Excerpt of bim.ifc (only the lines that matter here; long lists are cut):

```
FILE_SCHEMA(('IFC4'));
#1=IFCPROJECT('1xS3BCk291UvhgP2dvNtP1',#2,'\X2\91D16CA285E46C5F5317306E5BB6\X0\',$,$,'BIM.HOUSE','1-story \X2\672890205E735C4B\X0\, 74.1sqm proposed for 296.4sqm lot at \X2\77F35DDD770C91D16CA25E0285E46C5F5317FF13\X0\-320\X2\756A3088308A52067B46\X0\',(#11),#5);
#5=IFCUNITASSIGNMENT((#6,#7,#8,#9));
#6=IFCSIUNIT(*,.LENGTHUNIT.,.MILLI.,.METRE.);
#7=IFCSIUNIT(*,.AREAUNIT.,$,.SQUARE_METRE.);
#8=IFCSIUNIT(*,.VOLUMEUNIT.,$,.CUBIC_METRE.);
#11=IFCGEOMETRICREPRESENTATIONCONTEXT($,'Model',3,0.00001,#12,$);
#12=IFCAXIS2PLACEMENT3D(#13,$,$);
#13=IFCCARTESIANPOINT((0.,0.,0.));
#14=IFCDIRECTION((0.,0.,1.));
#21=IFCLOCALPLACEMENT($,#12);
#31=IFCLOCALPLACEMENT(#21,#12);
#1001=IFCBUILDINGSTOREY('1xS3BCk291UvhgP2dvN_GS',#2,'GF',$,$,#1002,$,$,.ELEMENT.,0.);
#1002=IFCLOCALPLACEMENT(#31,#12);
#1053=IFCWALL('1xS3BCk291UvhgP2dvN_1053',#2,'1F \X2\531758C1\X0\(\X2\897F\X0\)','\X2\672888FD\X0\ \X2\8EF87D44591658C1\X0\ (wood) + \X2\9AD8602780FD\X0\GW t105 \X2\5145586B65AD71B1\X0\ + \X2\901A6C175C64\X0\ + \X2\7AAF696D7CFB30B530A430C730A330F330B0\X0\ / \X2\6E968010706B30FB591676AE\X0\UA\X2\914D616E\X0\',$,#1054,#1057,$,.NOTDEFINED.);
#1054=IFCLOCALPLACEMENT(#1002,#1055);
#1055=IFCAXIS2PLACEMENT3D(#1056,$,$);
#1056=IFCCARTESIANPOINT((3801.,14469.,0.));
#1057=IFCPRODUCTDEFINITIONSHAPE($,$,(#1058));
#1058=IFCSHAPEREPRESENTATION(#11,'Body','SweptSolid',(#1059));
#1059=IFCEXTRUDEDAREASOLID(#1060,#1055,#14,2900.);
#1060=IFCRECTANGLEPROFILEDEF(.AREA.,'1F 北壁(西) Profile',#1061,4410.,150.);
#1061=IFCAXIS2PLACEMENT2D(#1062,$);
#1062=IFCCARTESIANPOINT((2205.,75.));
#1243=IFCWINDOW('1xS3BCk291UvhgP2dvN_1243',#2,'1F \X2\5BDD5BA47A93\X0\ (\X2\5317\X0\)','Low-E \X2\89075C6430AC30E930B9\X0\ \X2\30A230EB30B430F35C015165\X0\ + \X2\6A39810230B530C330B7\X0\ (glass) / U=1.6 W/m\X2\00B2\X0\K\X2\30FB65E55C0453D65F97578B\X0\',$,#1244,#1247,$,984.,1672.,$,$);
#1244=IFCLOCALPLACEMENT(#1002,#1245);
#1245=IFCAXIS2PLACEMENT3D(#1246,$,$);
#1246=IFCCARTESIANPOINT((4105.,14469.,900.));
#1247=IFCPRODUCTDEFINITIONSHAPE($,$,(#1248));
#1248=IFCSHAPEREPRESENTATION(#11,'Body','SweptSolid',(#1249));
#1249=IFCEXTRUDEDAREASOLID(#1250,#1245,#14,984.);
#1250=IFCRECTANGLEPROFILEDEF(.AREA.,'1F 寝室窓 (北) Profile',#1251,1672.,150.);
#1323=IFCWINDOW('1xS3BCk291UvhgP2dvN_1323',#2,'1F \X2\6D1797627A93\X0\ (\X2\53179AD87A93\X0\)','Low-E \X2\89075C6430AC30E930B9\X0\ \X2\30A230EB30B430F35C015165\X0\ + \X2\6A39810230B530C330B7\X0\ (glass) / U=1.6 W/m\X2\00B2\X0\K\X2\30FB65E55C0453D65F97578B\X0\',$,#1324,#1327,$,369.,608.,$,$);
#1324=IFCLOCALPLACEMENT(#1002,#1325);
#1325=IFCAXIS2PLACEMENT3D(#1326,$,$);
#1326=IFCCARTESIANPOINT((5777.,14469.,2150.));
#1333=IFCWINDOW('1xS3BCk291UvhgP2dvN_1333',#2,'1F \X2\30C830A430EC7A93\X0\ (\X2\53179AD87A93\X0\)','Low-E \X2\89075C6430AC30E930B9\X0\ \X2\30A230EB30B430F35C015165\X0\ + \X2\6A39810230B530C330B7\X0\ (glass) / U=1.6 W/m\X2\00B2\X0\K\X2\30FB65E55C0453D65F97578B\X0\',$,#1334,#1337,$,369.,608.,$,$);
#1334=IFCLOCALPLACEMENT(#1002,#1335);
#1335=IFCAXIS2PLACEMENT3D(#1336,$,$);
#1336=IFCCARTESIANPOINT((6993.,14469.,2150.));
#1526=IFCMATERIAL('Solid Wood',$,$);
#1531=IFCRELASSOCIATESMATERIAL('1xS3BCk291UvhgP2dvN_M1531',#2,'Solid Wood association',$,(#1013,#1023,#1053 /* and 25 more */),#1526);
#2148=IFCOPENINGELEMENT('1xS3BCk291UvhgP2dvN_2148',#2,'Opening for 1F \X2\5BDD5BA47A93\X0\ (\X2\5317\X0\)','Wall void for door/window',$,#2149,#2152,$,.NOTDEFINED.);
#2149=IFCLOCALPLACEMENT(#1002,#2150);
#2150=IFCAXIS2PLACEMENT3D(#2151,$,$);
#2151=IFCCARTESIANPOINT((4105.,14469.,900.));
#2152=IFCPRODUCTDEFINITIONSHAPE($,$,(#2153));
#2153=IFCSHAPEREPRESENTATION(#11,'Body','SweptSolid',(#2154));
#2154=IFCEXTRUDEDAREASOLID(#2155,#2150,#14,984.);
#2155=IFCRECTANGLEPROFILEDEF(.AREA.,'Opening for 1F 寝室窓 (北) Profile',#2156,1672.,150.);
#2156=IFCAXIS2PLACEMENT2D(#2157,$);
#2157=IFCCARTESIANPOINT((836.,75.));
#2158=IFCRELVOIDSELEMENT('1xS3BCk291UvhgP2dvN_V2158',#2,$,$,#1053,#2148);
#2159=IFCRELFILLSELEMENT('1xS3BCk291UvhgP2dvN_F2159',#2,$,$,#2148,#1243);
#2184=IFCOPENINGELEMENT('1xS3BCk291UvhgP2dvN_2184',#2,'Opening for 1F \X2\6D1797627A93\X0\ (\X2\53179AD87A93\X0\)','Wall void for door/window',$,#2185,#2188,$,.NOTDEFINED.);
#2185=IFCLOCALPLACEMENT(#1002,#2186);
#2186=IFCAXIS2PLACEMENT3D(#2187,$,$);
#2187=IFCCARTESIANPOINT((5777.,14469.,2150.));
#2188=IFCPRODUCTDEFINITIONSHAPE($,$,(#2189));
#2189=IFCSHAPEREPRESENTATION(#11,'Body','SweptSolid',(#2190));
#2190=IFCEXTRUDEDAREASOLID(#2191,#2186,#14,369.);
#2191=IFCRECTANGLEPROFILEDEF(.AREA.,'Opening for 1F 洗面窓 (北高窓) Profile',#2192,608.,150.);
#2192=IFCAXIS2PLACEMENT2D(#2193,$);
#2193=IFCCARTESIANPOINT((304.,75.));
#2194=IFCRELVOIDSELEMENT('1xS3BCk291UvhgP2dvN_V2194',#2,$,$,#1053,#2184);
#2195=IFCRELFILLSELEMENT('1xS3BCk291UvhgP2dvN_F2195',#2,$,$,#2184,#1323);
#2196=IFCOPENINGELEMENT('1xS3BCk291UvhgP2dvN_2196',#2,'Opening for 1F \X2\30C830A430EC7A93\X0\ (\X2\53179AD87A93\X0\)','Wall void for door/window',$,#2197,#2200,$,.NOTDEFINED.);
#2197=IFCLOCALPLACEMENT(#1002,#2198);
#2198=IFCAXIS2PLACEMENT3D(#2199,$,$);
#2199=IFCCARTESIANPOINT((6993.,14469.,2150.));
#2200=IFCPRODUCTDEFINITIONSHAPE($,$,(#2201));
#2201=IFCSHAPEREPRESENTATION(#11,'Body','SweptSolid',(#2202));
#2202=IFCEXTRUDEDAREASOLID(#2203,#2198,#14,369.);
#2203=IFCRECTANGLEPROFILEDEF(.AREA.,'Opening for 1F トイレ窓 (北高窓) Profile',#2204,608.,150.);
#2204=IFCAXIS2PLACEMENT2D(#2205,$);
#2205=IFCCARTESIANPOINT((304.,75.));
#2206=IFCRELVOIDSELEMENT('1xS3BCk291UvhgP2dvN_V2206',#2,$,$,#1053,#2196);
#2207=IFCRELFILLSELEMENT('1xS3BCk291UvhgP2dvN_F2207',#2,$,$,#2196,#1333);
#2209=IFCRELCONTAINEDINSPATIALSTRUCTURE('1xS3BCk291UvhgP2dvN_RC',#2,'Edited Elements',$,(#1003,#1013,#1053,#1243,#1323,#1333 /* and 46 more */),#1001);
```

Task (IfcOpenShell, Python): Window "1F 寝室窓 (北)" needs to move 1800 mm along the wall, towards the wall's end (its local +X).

```python
import ifcopenshell
import ifcopenshell.api.geometry
import ifcopenshell.util.placement

model = ifcopenshell.open("bim.ifc")

window = model.by_guid("1xS3BCk291UvhgP2dvN_1243")
opening = window.FillsVoids[0].RelatingOpeningElement
wall = opening.VoidsElements[0].RelatingBuildingElement

wall_matrix = ifcopenshell.util.placement.get_local_placement(wall.ObjectPlacement)
shift = wall_matrix[:3, 0] * 1800.0
before = ifcopenshell.util.placement.get_local_placement(window.ObjectPlacement)[:3, 3].copy()

# The window is not placed relative to its opening, so move both.
for product in (opening, window):
    matrix = ifcopenshell.util.placement.get_local_placement(product.ObjectPlacement)
    matrix[:3, 3] += shift
    ifcopenshell.api.geometry.edit_object_placement(model, product=product, matrix=matrix, is_si=False)

after = ifcopenshell.util.placement.get_local_placement(window.ObjectPlacement)[:3, 3]
print("window moved by", (after - before).round(3) + 0.0)

model.write("bim_updated.ifc")
```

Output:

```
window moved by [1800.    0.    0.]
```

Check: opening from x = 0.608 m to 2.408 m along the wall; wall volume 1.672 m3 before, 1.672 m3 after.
